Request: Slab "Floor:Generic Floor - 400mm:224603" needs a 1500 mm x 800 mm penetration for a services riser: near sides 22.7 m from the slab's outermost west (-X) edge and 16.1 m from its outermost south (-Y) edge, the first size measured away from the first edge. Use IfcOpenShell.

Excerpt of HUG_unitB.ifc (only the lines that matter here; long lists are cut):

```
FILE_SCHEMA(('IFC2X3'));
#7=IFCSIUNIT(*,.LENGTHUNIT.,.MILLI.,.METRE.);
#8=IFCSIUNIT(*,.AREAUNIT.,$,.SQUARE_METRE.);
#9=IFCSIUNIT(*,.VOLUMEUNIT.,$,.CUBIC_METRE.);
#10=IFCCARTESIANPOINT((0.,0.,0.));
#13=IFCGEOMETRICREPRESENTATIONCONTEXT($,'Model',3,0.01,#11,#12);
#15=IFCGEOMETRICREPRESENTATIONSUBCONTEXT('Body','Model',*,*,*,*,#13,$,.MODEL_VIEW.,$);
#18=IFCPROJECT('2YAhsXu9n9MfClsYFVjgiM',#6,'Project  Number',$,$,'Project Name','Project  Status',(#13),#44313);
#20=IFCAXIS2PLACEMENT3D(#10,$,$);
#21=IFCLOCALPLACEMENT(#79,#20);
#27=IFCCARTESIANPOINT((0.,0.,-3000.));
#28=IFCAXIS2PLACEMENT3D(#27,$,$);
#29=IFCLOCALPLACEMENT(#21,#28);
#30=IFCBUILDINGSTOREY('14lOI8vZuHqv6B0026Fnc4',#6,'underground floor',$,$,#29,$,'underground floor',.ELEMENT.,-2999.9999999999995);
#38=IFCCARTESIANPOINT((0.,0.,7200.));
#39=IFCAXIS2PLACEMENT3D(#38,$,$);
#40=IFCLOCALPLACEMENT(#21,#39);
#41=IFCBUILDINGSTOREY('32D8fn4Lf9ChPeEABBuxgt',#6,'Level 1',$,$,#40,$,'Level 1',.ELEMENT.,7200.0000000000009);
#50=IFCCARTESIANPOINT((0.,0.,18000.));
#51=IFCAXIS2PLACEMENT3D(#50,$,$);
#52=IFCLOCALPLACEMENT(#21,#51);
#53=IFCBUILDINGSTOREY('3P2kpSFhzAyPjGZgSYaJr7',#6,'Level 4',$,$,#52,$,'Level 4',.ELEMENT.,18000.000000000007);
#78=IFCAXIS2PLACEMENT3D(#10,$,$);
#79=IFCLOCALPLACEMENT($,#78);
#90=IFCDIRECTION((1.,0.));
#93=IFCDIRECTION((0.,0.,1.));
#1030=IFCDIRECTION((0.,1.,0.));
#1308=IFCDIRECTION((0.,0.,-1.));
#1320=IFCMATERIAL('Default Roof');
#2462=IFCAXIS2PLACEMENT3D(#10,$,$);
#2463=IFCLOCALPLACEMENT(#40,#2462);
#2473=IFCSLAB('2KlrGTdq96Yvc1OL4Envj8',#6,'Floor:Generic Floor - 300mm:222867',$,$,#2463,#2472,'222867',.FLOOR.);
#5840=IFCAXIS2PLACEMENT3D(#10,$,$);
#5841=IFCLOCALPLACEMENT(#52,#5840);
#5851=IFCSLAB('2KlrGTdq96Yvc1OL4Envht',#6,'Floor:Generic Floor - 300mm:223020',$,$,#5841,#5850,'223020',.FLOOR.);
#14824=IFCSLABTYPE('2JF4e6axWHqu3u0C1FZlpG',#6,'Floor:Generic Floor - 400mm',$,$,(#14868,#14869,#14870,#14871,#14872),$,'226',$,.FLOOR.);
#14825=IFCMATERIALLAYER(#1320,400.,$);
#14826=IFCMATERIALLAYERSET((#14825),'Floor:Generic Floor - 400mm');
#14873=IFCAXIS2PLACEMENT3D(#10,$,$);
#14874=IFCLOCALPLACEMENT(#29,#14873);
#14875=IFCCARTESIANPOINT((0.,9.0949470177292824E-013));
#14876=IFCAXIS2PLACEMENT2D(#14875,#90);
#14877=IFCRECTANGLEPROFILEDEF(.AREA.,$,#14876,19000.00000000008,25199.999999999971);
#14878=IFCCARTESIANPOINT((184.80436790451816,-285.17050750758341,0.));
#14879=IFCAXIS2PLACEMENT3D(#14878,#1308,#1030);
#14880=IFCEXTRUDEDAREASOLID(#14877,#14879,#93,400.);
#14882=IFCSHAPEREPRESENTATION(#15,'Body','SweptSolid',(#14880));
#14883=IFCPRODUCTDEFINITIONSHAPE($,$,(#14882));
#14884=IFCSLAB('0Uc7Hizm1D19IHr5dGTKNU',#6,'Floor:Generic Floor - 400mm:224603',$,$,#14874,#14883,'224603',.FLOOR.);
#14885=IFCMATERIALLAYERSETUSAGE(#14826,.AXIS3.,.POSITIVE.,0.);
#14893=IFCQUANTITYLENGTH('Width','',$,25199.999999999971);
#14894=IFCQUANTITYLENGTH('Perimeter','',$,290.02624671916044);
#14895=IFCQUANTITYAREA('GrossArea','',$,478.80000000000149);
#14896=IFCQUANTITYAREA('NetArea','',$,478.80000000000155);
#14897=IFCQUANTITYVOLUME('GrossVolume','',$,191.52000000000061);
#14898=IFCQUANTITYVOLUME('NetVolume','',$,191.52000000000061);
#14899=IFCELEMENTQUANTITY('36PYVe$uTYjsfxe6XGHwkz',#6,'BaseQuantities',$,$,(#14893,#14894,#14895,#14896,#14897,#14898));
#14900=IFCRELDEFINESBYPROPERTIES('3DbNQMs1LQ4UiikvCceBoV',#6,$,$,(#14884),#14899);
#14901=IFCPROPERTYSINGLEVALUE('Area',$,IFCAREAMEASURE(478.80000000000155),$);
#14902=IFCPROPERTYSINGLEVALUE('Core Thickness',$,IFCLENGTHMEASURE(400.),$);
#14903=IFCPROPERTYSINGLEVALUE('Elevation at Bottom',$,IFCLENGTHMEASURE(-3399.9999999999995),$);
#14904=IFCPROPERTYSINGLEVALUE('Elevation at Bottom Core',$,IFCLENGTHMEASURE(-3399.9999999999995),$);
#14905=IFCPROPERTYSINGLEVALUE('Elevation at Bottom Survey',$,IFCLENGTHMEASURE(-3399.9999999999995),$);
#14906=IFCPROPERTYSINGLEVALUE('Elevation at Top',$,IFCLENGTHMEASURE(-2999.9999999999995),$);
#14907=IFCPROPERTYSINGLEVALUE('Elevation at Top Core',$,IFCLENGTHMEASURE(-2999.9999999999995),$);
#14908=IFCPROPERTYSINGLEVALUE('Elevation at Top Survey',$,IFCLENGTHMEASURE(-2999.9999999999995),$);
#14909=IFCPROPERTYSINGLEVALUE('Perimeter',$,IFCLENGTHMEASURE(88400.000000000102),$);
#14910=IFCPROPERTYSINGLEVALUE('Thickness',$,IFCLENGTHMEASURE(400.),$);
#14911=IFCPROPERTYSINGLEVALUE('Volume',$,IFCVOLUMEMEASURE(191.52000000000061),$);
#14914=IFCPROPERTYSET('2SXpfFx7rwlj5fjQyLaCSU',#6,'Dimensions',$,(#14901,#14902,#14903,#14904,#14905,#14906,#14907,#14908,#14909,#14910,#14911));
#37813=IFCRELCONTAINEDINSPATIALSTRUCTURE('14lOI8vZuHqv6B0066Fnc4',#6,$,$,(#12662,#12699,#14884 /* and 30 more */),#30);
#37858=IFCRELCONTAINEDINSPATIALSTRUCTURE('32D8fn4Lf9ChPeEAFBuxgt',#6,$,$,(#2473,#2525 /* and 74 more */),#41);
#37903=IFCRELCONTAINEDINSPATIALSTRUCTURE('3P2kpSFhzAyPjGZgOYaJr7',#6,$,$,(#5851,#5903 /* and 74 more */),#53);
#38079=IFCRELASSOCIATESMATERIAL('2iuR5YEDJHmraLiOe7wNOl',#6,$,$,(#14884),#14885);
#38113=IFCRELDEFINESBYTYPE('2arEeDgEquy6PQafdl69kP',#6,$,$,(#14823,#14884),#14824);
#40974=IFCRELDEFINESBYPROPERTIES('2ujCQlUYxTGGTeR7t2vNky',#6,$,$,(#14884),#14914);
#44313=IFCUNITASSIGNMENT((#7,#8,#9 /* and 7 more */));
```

```python
import numpy as np
import ifcopenshell
import ifcopenshell.api.feature
import ifcopenshell.api.geometry
import ifcopenshell.api.pset
import ifcopenshell.api.root
import ifcopenshell.geom
import ifcopenshell.util.element
import ifcopenshell.util.placement
import ifcopenshell.util.representation
import ifcopenshell.util.shape
import ifcopenshell.util.unit

model = ifcopenshell.open("HUG_unitB.ifc")
unit_scale = ifcopenshell.util.unit.calculate_unit_scale(model)
area_scale = ifcopenshell.util.unit.calculate_unit_scale(model, "AREAUNIT")
volume_scale = ifcopenshell.util.unit.calculate_unit_scale(model, "VOLUMEUNIT")
settings = ifcopenshell.geom.settings()


def volume(element):
    """Net volume in cubic metres, openings subtracted."""
    shape = ifcopenshell.geom.create_shape(settings, element)
    return ifcopenshell.util.shape.get_volume(shape.geometry)


slab = model.by_guid("0Uc7Hizm1D19IHr5dGTKNU")
before = volume(slab)

# Extent in the slab's own axes, in metres. The edges named are its -X and -Y sides.
slab_shape = ifcopenshell.geom.create_shape(settings, slab)
vertices = ifcopenshell.util.shape.get_vertices(slab_shape.geometry)
x_min, y_min, bottom = vertices.min(axis=0)
top = vertices[:, 2].max()

opening = ifcopenshell.api.root.create_entity(model, ifc_class="IfcOpeningElement", name="Services riser opening")
context = ifcopenshell.util.representation.get_context(model, "Model", "Body", "MODEL_VIEW")
width, depth = 1.5, 0.8
outline = [(0.0, 0.0), (width, 0.0), (width, depth), (0.0, depth), (0.0, 0.0)]
# Overshoot both faces by 50 mm so the cut is clean.
shape = ifcopenshell.api.geometry.add_slab_representation(
    model, context=context, depth=top - bottom + 0.1, polyline=outline
)
ifcopenshell.api.geometry.assign_representation(model, product=opening, representation=shape)

matrix = ifcopenshell.util.placement.get_local_placement(slab.ObjectPlacement)
matrix[:, 3] = matrix @ np.append(np.array([x_min + 22.7, y_min + 16.1, bottom - 0.05]) / unit_scale, 1.0)
ifcopenshell.api.geometry.edit_object_placement(model, product=opening, matrix=matrix, is_si=False)
ifcopenshell.api.feature.add_feature(model, feature=opening, element=slab)

after = volume(slab)

# Update the slab's stored quantities.
qto = model.by_id(ifcopenshell.util.element.get_pset(slab, "BaseQuantities", should_inherit=False)["id"])
ifcopenshell.api.pset.edit_qto(model, qto=qto, properties={
    "NetArea": after / (top - bottom) / area_scale,
    "NetVolume": after / volume_scale,
})
pset = model.by_id(ifcopenshell.util.element.get_pset(slab, "Dimensions", should_inherit=False)["id"])
ifcopenshell.api.pset.edit_pset(model, pset=pset, properties={
    "Area": model.create_entity("IfcAreaMeasure", after / (top - bottom) / area_scale),
    "Volume": model.create_entity("IfcVolumeMeasure", after / volume_scale),
})

print(f"slab volume {before:.3f} -> {after:.3f} m3")

model.write("HUG_unitB_v2.ifc")
```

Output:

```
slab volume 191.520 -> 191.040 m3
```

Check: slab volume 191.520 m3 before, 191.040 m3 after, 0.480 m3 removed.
